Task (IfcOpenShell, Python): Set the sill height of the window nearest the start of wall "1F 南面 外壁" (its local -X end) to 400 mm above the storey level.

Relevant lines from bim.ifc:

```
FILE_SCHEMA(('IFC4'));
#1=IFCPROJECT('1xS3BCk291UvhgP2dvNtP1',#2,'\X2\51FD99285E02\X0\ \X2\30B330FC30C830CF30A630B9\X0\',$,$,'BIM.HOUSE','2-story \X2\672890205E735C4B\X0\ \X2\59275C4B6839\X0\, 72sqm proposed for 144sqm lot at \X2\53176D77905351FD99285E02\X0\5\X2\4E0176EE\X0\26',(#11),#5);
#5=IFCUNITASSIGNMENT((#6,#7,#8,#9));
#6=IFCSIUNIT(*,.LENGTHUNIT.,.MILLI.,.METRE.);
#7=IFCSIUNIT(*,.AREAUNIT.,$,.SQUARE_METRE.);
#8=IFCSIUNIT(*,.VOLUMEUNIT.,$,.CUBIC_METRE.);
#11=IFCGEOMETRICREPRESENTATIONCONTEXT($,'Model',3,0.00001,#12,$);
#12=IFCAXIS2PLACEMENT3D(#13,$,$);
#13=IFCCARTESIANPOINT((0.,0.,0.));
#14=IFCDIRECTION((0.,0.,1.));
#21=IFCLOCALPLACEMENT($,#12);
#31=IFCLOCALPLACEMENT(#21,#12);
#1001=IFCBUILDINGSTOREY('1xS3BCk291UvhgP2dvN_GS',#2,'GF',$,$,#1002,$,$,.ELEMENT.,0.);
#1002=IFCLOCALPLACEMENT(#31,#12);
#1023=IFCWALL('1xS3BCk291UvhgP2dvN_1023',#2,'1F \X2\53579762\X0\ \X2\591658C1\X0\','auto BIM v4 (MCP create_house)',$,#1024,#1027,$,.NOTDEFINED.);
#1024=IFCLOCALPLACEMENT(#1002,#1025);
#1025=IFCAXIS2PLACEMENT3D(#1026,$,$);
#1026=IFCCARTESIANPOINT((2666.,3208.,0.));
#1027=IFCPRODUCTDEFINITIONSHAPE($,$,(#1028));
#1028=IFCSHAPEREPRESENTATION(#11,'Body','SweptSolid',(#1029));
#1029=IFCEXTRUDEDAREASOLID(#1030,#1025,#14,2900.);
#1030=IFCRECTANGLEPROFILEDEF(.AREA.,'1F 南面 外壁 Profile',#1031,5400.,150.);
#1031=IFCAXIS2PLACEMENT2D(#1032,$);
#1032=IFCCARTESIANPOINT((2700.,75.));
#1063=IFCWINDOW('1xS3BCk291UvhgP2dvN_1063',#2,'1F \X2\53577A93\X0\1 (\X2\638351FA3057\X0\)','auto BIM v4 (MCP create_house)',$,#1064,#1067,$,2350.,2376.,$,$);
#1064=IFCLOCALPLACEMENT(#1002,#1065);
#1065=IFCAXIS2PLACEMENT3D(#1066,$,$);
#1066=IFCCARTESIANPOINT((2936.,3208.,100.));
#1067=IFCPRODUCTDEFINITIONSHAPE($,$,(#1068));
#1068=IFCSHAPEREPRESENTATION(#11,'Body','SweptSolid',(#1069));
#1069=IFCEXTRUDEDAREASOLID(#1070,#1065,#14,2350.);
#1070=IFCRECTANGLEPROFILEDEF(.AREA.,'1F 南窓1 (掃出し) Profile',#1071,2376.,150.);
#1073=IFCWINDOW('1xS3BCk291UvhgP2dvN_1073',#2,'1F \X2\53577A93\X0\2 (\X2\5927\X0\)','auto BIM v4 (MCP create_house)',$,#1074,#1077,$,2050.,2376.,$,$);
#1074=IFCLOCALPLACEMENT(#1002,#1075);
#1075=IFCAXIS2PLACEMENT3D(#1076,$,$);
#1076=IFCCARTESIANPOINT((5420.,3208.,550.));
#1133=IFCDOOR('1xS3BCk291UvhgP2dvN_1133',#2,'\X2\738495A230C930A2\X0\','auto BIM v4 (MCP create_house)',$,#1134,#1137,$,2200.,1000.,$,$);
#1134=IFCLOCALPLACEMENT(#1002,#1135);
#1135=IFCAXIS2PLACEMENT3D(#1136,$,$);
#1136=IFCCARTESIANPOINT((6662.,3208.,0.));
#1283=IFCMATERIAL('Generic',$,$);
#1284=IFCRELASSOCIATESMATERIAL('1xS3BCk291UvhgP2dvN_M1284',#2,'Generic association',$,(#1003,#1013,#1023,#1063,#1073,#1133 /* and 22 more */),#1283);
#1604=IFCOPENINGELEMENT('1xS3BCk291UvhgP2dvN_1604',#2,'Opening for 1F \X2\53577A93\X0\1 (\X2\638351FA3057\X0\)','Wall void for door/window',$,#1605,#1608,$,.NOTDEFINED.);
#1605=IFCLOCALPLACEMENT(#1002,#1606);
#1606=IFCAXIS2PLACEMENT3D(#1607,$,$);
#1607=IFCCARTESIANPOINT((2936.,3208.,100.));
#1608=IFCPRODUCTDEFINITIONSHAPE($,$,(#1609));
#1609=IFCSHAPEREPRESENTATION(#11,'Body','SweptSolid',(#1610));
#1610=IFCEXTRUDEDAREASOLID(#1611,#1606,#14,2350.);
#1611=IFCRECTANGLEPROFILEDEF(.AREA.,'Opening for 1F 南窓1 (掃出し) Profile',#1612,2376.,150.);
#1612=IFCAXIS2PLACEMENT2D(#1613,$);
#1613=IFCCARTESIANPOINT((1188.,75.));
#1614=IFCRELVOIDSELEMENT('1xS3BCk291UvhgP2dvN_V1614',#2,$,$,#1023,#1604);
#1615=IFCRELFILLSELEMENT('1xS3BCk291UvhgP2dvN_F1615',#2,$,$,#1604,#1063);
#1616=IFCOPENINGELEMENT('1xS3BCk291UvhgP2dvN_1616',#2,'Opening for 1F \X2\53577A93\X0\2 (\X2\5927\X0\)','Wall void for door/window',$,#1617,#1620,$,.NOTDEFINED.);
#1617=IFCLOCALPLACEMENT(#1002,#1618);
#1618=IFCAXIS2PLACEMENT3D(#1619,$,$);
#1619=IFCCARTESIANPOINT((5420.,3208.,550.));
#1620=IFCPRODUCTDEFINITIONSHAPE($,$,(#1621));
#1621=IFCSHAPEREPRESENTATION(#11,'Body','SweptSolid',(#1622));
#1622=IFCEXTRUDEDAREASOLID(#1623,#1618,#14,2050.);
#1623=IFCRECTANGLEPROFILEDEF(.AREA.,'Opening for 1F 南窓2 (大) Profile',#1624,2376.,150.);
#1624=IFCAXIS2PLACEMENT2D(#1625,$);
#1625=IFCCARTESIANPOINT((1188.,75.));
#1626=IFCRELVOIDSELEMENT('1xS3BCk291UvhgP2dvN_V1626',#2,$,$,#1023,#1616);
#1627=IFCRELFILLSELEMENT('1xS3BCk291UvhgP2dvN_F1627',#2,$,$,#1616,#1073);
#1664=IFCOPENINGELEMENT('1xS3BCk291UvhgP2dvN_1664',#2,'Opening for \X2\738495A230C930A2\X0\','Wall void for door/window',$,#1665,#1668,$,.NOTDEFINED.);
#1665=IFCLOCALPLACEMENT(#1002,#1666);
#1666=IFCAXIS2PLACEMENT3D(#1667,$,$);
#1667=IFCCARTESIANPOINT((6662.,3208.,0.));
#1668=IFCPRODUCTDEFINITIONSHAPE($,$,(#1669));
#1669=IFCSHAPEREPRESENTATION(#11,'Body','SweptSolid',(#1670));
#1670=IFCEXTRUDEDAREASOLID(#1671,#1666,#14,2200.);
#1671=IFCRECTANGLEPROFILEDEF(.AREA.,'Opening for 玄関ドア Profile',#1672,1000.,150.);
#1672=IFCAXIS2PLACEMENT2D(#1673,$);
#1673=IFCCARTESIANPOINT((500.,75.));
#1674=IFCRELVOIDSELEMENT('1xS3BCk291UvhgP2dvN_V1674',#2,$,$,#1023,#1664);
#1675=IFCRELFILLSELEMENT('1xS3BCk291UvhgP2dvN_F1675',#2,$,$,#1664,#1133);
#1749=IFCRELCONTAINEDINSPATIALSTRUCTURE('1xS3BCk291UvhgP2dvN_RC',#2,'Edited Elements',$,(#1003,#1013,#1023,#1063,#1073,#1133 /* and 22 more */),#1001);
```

```python
import numpy as np
import ifcopenshell
import ifcopenshell.api.geometry
import ifcopenshell.geom
import ifcopenshell.util.element
import ifcopenshell.util.placement
import ifcopenshell.util.shape
import ifcopenshell.util.unit

model = ifcopenshell.open("bim.ifc")
unit_scale = ifcopenshell.util.unit.calculate_unit_scale(model)

window = model.by_id(1063)
opening = window.FillsVoids[0].RelatingOpeningElement
storey = ifcopenshell.util.element.get_container(window, ifc_class="IfcBuildingStorey")
level = ifcopenshell.util.placement.get_local_placement(storey.ObjectPlacement)[2, 3]

# The opening's origin need not be at the sill, so measure its lowest point.
shape = ifcopenshell.geom.create_shape(ifcopenshell.geom.settings(), opening)
bottom = ifcopenshell.util.shape.get_shape_bottom_elevation(shape, shape.geometry) / unit_scale
dz = level + 0.4 / unit_scale - bottom

shift = np.array([0.0, 0.0, dz])
# The window is not placed relative to its opening, so move both.
for product in (opening, window):
    matrix = ifcopenshell.util.placement.get_local_placement(product.ObjectPlacement)
    matrix[:3, 3] += shift
    ifcopenshell.api.geometry.edit_object_placement(model, product=product, matrix=matrix, is_si=False)

print(f"moved by {dz * unit_scale:+.3f} m")

model.write("bim_edited.ifc")
```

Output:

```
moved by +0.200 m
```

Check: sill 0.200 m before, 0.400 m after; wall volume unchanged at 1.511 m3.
